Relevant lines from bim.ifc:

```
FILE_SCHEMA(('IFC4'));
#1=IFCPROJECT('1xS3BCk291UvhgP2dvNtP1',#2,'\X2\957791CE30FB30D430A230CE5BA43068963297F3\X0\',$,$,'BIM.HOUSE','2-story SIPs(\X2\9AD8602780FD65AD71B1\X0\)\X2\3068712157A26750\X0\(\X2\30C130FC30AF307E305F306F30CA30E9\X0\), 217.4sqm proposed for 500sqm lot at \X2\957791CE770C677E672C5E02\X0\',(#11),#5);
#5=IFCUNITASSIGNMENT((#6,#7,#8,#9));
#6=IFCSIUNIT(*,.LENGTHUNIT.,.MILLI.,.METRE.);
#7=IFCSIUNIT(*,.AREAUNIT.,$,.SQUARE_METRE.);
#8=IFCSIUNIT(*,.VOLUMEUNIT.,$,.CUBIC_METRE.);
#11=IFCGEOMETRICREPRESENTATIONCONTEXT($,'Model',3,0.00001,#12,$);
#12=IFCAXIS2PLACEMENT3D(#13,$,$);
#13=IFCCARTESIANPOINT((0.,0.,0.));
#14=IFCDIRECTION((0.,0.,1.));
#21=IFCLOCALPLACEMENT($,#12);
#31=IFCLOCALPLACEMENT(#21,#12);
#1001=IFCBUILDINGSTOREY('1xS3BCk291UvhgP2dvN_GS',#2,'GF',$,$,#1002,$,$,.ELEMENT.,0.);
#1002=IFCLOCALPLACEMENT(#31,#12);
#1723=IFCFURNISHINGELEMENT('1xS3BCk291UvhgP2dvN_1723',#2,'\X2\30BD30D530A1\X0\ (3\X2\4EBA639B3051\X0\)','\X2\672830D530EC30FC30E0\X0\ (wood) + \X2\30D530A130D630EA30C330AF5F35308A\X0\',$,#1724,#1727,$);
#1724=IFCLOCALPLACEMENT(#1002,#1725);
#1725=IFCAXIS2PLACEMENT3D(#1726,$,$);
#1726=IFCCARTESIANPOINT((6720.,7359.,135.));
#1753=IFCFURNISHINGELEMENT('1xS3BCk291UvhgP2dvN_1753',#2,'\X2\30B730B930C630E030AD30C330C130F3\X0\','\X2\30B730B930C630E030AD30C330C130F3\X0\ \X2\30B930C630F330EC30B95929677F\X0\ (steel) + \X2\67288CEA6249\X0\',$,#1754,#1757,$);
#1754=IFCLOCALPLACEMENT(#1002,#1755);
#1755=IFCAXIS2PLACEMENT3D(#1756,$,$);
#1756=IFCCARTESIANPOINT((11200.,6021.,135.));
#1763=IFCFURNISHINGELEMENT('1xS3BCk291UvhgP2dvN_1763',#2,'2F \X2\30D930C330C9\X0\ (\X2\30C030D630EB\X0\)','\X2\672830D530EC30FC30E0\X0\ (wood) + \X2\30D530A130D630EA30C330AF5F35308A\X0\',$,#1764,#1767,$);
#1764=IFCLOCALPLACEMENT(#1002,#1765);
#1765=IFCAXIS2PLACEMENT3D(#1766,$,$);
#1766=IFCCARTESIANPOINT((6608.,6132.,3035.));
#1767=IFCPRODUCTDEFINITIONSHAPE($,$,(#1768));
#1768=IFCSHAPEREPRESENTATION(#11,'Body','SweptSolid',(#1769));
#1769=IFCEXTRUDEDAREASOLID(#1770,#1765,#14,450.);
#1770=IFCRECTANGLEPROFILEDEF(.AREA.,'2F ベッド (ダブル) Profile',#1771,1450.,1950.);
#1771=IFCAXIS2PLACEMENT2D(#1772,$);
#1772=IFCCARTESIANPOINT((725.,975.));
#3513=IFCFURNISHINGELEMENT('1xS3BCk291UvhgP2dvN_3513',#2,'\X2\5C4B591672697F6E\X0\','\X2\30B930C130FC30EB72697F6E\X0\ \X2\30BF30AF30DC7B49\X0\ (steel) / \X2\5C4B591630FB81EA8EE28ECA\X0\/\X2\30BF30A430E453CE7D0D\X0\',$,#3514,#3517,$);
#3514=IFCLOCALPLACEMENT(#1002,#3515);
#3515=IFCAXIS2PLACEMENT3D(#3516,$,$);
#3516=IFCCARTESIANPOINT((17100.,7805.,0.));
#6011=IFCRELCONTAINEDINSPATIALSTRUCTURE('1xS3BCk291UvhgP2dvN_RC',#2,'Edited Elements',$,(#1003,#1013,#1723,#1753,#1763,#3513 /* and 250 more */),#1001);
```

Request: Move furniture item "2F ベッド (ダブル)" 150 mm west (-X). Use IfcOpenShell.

```python
import ifcopenshell
import ifcopenshell.api.geometry
import ifcopenshell.util.placement
import ifcopenshell.util.unit

model = ifcopenshell.open("bim.ifc")
unit_scale = ifcopenshell.util.unit.calculate_unit_scale(model)

item = model.by_id(1763)
matrix = ifcopenshell.util.placement.get_local_placement(item.ObjectPlacement)
matrix[0, 3] -= 0.15 / unit_scale
ifcopenshell.api.geometry.edit_object_placement(model, product=item, matrix=matrix, is_si=False)

print(ifcopenshell.util.placement.get_local_placement(item.ObjectPlacement).round(3) + 0.0)

model.write("bim_updated.ifc")
```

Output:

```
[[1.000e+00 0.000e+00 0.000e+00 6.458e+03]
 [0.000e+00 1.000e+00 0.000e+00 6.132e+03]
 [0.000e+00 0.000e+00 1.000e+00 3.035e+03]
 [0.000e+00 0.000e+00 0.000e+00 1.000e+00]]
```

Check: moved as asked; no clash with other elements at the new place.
